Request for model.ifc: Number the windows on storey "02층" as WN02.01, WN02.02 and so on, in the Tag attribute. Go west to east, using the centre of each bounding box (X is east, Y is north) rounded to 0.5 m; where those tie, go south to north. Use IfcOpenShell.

First a look at what the model holds.

```python
import ifcopenshell
import ifcopenshell.util.element
import ifcopenshell.util.placement

model = ifcopenshell.open("model.ifc")
print(model.schema)
storey = next(s for s in model.by_type("IfcBuildingStorey") if s.Name == "02층")
windows = [e for e in ifcopenshell.util.element.get_decomposition(storey) if e.is_a("IfcWindow")]
for e in sorted(windows, key=lambda e: e.id()):
    origin = ifcopenshell.util.placement.get_local_placement(e.ObjectPlacement)[:3, 3]
    print(e.id(), e.Tag, e.Name, origin.round(2) + 0.0, sep=" | ")
```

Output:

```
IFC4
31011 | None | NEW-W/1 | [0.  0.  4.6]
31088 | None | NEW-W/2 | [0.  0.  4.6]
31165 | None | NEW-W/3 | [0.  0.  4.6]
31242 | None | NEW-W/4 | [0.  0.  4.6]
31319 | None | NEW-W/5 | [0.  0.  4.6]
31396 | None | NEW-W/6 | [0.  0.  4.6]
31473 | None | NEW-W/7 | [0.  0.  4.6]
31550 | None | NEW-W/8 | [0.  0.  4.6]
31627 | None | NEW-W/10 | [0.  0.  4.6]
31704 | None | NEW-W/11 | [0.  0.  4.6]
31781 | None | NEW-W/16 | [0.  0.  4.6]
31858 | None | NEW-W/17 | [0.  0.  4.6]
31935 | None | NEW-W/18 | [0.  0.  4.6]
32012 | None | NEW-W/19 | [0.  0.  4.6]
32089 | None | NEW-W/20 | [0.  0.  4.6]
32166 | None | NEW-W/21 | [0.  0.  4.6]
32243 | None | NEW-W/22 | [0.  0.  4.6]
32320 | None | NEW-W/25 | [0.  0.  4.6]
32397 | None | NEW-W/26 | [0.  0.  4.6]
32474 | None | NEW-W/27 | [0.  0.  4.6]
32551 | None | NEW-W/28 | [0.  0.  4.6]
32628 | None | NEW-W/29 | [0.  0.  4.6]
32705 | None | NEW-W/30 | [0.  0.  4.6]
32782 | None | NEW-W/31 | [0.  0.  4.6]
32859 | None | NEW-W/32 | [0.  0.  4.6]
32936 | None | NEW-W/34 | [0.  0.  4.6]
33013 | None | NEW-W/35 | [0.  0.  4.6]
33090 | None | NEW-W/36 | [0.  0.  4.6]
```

```python
import ifcopenshell
import ifcopenshell.geom
import ifcopenshell.util.element
import ifcopenshell.util.shape

model = ifcopenshell.open("model.ifc")
settings = ifcopenshell.geom.settings()
settings.set("use-world-coords", True)


def centre(element):
    shape = ifcopenshell.geom.create_shape(settings, element)
    return ifcopenshell.util.shape.get_bbox_centroid(shape.geometry)


storey = next(s for s in model.by_type("IfcBuildingStorey") if s.Name == "02층")
windows = [e for e in ifcopenshell.util.element.get_decomposition(storey) if e.is_a("IfcWindow")]

# Insertion points can sit at a corner or the storey origin, so sort by the geometry (in metres).
centres = {e: centre(e) for e in windows}
windows.sort(key=lambda e: (round(centres[e][0] / 0.5), centres[e][1]))

for i, e in enumerate(windows, start=1):
    number = f"WN02.{i:02d}"
    e.Tag = number
    print(e.id(), number)

model.write("model_rev.ifc")
```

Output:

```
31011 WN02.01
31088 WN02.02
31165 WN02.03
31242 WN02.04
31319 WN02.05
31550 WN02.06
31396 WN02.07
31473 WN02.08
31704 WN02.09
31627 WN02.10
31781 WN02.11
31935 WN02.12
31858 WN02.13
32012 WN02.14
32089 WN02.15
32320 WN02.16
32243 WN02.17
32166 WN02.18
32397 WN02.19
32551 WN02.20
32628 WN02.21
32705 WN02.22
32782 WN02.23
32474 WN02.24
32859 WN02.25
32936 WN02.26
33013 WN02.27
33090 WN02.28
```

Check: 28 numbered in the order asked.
